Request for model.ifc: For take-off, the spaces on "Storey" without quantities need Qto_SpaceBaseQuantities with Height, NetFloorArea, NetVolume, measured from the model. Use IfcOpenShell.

First a look at what the model holds.

```python
import ifcopenshell
import ifcopenshell.util.element
import ifcopenshell.util.unit

model = ifcopenshell.open("model.ifc")
print(model.schema)
for unit_type in ("LENGTHUNIT", "AREAUNIT", "VOLUMEUNIT"):
    print(unit_type, ifcopenshell.util.unit.calculate_unit_scale(model, unit_type))
storey = next(s for s in model.by_type("IfcBuildingStorey") if s.Name == "Storey")
spaces = [e for e in ifcopenshell.util.element.get_decomposition(storey) if e.is_a("IfcSpace")]
for e in sorted(spaces, key=lambda e: e.id()):
    print(e.id(), e.is_a(), e.Name, list(ifcopenshell.util.element.get_psets(e, qtos_only=True)), sep=" | ")
```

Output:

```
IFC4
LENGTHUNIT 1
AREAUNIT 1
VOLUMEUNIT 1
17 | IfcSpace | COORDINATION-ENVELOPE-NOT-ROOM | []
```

```python
import ifcopenshell
import ifcopenshell.api.pset
import ifcopenshell.geom
import ifcopenshell.util.element
import ifcopenshell.util.shape
import ifcopenshell.util.unit

model = ifcopenshell.open("model.ifc")
unit_scale = ifcopenshell.util.unit.calculate_unit_scale(model)
area_scale = ifcopenshell.util.unit.calculate_unit_scale(model, "AREAUNIT")
volume_scale = ifcopenshell.util.unit.calculate_unit_scale(model, "VOLUMEUNIT")
settings = ifcopenshell.geom.settings()

storey = next(s for s in model.by_type("IfcBuildingStorey") if s.Name == "Storey")
spaces = [e for e in ifcopenshell.util.element.get_decomposition(storey) if e.is_a("IfcSpace")]

for e in sorted(spaces, key=lambda e: e.id()):
    if ifcopenshell.util.element.get_psets(e, qtos_only=True, should_inherit=False):
        continue
    # Geometry comes back in metres, in the element's own axes.
    shape = ifcopenshell.geom.create_shape(settings, e)
    values = {
        "Height": ifcopenshell.util.shape.get_z(shape.geometry) / unit_scale,
        "NetFloorArea": ifcopenshell.util.shape.get_footprint_area(shape.geometry) / area_scale,
        "NetVolume": ifcopenshell.util.shape.get_volume(shape.geometry) / volume_scale,
    }
    qto = ifcopenshell.api.pset.add_qto(model, product=e, name="Qto_SpaceBaseQuantities")
    ifcopenshell.api.pset.edit_qto(model, qto=qto, properties=values)
    print(e.id(), {k: round(v, 3) for k, v in values.items()})

model.write("model_updated.ifc")
```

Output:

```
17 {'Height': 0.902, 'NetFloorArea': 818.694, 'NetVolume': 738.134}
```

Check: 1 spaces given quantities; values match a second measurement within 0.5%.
